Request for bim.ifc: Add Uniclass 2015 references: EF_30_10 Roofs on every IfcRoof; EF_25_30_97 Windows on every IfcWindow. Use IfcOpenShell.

First a look at what the model holds.

```python
import ifcopenshell

model = ifcopenshell.open("bim.ifc")
print(model.schema)
print("classifications:", [c.Name for c in model.by_type("IfcClassification")])
for ifc_class in ("IfcDoor", "IfcRoof", "IfcStair", "IfcWall", "IfcWindow"):
    print(ifc_class, len(model.by_type(ifc_class)))
```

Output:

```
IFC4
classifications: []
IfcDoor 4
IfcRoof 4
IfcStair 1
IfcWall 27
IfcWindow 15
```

```python
import ifcopenshell
import ifcopenshell.api.classification

model = ifcopenshell.open("bim.ifc")

system = ifcopenshell.api.classification.add_classification(model, classification="Uniclass 2015")

codes = {
    "IfcRoof": ("EF_30_10", "Roofs"),
    "IfcWindow": ("EF_25_30_97", "Windows"),
}
for ifc_class, (code, name) in codes.items():
    products = model.by_type(ifc_class)
    ifcopenshell.api.classification.add_reference(
        model, products=products, classification=system, identification=code, name=name
    )
    print(code, len(products))

model.write("bim_updated.ifc")
```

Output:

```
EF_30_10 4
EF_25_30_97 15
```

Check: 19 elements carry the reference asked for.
